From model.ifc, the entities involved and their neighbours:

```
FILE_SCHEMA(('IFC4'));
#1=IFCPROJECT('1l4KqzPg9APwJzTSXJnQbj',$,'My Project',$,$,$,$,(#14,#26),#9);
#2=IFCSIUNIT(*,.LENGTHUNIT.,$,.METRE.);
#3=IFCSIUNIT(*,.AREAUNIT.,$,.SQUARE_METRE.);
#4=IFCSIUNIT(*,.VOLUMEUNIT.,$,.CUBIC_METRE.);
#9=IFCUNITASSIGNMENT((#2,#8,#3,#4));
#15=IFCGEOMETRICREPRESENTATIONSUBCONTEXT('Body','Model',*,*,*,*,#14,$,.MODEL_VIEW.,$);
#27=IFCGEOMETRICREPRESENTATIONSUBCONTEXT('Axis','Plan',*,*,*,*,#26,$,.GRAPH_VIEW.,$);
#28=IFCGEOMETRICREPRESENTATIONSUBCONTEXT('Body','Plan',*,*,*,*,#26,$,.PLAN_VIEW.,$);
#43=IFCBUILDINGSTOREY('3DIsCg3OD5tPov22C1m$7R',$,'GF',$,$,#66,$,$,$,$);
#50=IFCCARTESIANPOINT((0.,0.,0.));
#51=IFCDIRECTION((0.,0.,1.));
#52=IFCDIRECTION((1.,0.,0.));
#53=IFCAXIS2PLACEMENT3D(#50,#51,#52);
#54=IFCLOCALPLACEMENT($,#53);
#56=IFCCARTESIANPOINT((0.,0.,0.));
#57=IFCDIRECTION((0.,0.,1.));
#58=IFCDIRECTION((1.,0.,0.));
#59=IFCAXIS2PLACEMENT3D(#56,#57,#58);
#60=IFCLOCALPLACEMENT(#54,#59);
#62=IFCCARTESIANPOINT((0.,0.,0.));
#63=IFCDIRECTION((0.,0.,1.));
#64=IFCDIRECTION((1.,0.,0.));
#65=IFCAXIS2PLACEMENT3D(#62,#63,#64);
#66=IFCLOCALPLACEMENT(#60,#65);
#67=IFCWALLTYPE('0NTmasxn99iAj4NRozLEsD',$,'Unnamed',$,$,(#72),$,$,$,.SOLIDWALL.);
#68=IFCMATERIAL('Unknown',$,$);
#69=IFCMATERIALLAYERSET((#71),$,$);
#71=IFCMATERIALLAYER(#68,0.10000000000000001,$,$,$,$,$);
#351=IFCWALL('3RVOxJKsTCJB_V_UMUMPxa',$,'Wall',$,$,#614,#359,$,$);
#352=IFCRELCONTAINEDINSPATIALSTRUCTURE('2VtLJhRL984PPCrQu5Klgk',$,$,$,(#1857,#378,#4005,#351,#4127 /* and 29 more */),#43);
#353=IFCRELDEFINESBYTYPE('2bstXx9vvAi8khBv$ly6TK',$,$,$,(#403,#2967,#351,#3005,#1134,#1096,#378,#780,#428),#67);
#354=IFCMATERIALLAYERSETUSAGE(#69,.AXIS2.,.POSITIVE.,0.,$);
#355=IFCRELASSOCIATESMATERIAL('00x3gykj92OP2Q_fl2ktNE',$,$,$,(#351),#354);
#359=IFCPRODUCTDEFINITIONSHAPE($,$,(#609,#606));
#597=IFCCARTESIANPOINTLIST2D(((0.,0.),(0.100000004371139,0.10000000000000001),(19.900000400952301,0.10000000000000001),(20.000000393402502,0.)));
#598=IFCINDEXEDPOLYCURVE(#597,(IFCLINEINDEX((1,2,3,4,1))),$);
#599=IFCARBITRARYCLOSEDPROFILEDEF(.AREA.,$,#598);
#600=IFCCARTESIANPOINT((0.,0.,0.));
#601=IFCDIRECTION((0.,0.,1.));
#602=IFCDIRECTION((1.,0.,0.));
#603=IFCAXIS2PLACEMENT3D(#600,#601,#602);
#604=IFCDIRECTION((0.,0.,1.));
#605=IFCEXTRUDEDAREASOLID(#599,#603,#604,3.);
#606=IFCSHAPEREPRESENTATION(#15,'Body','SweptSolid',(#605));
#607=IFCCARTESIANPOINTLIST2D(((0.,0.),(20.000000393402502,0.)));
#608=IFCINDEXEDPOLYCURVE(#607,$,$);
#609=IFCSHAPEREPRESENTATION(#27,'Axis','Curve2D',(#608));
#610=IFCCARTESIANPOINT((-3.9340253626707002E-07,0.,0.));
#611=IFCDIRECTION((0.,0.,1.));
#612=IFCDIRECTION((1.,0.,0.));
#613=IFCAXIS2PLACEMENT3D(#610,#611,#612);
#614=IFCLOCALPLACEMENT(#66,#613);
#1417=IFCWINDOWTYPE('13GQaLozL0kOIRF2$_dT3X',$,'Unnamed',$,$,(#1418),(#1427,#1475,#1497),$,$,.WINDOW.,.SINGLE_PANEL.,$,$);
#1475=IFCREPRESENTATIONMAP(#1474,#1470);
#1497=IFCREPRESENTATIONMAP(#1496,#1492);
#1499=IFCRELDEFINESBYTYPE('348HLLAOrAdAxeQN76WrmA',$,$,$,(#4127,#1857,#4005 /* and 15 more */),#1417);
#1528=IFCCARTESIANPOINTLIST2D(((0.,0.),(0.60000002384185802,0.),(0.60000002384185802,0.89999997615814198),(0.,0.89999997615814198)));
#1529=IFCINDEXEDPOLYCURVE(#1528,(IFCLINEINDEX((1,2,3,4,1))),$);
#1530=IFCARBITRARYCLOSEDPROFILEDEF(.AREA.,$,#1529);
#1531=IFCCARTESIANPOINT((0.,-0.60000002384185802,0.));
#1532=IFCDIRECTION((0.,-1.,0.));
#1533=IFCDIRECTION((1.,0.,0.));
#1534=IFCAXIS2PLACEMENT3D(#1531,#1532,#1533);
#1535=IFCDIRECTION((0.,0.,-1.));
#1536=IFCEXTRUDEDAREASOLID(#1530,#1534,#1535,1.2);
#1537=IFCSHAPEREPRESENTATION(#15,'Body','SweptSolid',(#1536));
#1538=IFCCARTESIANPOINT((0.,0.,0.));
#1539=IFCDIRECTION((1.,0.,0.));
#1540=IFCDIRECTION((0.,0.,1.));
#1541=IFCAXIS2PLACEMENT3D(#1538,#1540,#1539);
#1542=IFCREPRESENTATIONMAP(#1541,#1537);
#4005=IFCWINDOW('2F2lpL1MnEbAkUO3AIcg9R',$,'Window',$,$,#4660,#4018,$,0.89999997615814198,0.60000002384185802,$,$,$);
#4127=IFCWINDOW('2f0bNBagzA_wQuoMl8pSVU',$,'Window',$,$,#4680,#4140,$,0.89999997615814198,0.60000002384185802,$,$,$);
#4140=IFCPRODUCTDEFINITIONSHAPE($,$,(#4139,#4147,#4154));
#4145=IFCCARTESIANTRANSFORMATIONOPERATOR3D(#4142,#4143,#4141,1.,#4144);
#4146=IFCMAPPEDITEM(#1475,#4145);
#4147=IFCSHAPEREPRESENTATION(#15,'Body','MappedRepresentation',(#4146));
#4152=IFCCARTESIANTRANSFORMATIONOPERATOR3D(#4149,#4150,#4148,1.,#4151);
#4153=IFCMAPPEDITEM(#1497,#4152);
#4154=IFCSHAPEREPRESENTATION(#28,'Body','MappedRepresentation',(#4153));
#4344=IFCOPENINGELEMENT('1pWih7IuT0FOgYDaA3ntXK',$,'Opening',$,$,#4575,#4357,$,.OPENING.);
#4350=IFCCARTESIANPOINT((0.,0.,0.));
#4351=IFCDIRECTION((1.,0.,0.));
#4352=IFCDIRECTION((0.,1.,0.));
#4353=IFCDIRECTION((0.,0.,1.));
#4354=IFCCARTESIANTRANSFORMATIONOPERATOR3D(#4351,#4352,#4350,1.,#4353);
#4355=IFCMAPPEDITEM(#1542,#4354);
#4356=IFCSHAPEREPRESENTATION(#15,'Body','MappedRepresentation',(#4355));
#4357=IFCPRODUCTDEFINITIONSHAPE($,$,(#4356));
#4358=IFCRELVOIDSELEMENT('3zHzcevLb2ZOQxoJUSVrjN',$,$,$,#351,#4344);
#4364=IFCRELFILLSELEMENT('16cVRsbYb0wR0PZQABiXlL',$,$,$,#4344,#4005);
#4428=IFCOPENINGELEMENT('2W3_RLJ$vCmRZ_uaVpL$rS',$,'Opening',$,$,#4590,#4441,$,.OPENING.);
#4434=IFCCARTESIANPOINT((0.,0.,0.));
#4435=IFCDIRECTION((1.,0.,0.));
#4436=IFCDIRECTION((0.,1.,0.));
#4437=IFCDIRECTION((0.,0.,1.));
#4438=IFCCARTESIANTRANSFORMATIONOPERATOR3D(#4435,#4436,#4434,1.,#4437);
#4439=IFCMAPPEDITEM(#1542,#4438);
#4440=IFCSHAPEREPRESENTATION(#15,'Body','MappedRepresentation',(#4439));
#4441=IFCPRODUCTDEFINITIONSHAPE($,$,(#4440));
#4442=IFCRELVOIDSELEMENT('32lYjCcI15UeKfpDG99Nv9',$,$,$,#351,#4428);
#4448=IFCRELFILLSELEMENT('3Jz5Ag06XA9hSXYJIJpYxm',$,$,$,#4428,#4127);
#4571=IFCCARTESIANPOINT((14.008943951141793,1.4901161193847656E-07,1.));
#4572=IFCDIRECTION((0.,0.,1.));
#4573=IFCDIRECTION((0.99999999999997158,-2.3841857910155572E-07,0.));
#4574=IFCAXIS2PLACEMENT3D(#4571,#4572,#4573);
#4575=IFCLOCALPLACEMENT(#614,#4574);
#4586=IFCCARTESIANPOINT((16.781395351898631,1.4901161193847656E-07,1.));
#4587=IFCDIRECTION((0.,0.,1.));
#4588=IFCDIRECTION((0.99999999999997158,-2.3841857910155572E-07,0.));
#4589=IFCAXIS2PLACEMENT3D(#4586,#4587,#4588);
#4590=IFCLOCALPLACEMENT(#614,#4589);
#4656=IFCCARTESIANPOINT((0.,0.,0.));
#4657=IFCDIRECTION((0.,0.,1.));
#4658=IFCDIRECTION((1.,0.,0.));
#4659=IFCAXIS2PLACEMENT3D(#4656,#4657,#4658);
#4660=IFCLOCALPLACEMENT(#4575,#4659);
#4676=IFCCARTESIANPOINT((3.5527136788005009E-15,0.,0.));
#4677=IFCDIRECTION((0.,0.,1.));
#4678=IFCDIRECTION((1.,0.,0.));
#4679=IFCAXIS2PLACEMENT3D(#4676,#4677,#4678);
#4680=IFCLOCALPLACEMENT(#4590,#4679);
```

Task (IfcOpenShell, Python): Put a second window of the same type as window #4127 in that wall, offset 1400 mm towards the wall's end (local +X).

```python
import ifcopenshell
import ifcopenshell.api.feature
import ifcopenshell.api.geometry
import ifcopenshell.api.root
import ifcopenshell.geom
import ifcopenshell.util.element
import ifcopenshell.util.placement
import ifcopenshell.util.shape
import ifcopenshell.util.unit

model = ifcopenshell.open("model.ifc")
unit_scale = ifcopenshell.util.unit.calculate_unit_scale(model)
settings = ifcopenshell.geom.settings()


def volume(element):
    """Net volume in cubic metres, openings subtracted."""
    shape = ifcopenshell.geom.create_shape(settings, element)
    return ifcopenshell.util.shape.get_volume(shape.geometry)


window = model.by_id(4127)
opening = window.FillsVoids[0].RelatingOpeningElement
wall = opening.VoidsElements[0].RelatingBuildingElement
before = volume(wall)
shift = ifcopenshell.util.placement.get_local_placement(wall.ObjectPlacement)[:3, 0] * 1.4 / unit_scale

# copy_class copies the void relationship, type, container and properties, but no geometry.
new_opening = ifcopenshell.api.root.copy_class(model, product=opening)
new_opening.Representation = ifcopenshell.util.element.copy_deep(
    model, opening.Representation, exclude=["IfcGeometricRepresentationContext", "IfcRepresentationMap"]
)
new_window = ifcopenshell.api.root.copy_class(model, product=window)
new_window.Representation = ifcopenshell.util.element.copy_deep(
    model, window.Representation, exclude=["IfcGeometricRepresentationContext", "IfcRepresentationMap"]
)
ifcopenshell.api.feature.add_filling(model, opening=new_opening, element=new_window)

for old, new in ((opening, new_opening), (window, new_window)):
    matrix = ifcopenshell.util.placement.get_local_placement(old.ObjectPlacement)
    matrix[:3, 3] += shift
    ifcopenshell.api.geometry.edit_object_placement(model, product=new, matrix=matrix, is_si=False)

after = volume(wall)

print(f"wall volume {before:.3f} -> {after:.3f} m3")

model.write("model-out.ifc")
```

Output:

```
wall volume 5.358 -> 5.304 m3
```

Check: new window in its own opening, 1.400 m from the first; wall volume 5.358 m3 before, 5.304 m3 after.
